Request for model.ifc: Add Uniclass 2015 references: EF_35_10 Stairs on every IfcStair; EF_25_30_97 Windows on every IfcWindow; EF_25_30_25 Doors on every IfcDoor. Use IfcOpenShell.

First a look at what the model holds.

```python
import ifcopenshell

model = ifcopenshell.open("model.ifc")
print(model.schema)
print("classifications:", [c.Name for c in model.by_type("IfcClassification")])
for ifc_class in ("IfcDoor", "IfcRoof", "IfcStair", "IfcWall", "IfcWindow"):
    print(ifc_class, len(model.by_type(ifc_class)))
```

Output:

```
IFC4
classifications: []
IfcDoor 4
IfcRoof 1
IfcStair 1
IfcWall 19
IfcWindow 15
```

```python
import ifcopenshell
import ifcopenshell.api.classification

model = ifcopenshell.open("model.ifc")

system = ifcopenshell.api.classification.add_classification(model, classification="Uniclass 2015")

codes = {
    "IfcStair": ("EF_35_10", "Stairs"),
    "IfcWindow": ("EF_25_30_97", "Windows"),
    "IfcDoor": ("EF_25_30_25", "Doors"),
}
for ifc_class, (code, name) in codes.items():
    products = model.by_type(ifc_class)
    ifcopenshell.api.classification.add_reference(
        model, products=products, classification=system, identification=code, name=name
    )
    print(code, len(products))

model.write("model_edited.ifc")
```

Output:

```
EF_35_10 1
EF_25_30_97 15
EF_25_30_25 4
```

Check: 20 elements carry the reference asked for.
